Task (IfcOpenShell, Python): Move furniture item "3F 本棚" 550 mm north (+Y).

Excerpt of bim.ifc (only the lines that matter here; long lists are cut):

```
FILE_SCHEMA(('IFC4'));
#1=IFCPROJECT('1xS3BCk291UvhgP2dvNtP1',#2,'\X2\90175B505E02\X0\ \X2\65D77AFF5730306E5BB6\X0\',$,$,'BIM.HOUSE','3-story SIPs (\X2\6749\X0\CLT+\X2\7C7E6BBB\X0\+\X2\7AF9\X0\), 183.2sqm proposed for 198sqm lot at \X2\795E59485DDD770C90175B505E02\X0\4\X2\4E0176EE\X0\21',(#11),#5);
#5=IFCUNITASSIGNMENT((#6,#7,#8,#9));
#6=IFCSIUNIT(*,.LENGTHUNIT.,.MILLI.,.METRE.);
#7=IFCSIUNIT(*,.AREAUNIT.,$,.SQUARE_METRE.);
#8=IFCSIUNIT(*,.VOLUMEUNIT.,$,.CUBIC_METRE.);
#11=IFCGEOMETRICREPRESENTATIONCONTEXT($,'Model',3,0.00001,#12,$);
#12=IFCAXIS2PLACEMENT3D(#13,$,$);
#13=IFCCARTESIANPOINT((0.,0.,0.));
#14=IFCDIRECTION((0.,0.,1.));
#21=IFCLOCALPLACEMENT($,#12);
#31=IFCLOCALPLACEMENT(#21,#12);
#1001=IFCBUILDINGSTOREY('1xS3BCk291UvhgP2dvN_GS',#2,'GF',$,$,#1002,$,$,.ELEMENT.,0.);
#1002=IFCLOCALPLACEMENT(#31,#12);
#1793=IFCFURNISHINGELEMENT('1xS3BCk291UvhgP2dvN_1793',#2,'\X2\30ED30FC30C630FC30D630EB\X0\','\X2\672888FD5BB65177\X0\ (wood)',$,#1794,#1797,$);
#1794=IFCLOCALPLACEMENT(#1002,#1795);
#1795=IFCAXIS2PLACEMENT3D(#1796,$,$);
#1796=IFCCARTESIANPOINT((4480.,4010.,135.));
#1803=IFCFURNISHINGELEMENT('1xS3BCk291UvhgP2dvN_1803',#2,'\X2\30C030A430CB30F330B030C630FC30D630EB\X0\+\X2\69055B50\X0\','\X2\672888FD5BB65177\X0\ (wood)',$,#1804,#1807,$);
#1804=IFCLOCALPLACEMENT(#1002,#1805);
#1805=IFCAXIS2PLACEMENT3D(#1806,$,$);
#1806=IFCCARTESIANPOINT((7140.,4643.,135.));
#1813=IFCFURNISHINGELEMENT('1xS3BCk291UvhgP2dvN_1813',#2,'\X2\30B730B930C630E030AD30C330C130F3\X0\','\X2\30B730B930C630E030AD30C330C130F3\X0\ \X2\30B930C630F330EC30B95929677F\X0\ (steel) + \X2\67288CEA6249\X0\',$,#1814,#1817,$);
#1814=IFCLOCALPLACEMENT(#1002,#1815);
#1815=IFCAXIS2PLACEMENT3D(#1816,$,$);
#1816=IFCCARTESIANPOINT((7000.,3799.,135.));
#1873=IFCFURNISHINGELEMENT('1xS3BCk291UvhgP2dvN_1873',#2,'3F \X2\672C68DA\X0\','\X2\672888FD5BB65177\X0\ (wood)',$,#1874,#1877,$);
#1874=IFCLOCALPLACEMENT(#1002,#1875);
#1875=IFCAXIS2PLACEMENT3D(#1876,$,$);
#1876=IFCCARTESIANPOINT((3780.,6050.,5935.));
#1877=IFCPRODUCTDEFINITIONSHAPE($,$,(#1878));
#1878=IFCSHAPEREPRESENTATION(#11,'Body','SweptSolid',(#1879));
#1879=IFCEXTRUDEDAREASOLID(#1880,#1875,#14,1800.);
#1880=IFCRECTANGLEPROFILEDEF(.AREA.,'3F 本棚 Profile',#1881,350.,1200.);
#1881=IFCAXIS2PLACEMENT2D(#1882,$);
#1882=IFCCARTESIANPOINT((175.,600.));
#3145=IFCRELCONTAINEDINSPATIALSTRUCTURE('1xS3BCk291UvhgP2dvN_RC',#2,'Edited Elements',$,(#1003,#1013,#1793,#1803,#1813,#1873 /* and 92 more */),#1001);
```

```python
import ifcopenshell
import ifcopenshell.api.geometry
import ifcopenshell.util.placement
import ifcopenshell.util.unit

model = ifcopenshell.open("bim.ifc")
unit_scale = ifcopenshell.util.unit.calculate_unit_scale(model)

item = model.by_guid("1xS3BCk291UvhgP2dvN_1873")
matrix = ifcopenshell.util.placement.get_local_placement(item.ObjectPlacement)
matrix[1, 3] += 0.55 / unit_scale
ifcopenshell.api.geometry.edit_object_placement(model, product=item, matrix=matrix, is_si=False)

print(ifcopenshell.util.placement.get_local_placement(item.ObjectPlacement).round(3) + 0.0)

model.write("bim_v2.ifc")
```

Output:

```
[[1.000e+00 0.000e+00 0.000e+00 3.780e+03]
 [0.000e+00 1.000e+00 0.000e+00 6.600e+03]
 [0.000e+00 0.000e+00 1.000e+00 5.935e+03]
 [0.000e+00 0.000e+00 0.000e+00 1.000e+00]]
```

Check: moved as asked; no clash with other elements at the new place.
